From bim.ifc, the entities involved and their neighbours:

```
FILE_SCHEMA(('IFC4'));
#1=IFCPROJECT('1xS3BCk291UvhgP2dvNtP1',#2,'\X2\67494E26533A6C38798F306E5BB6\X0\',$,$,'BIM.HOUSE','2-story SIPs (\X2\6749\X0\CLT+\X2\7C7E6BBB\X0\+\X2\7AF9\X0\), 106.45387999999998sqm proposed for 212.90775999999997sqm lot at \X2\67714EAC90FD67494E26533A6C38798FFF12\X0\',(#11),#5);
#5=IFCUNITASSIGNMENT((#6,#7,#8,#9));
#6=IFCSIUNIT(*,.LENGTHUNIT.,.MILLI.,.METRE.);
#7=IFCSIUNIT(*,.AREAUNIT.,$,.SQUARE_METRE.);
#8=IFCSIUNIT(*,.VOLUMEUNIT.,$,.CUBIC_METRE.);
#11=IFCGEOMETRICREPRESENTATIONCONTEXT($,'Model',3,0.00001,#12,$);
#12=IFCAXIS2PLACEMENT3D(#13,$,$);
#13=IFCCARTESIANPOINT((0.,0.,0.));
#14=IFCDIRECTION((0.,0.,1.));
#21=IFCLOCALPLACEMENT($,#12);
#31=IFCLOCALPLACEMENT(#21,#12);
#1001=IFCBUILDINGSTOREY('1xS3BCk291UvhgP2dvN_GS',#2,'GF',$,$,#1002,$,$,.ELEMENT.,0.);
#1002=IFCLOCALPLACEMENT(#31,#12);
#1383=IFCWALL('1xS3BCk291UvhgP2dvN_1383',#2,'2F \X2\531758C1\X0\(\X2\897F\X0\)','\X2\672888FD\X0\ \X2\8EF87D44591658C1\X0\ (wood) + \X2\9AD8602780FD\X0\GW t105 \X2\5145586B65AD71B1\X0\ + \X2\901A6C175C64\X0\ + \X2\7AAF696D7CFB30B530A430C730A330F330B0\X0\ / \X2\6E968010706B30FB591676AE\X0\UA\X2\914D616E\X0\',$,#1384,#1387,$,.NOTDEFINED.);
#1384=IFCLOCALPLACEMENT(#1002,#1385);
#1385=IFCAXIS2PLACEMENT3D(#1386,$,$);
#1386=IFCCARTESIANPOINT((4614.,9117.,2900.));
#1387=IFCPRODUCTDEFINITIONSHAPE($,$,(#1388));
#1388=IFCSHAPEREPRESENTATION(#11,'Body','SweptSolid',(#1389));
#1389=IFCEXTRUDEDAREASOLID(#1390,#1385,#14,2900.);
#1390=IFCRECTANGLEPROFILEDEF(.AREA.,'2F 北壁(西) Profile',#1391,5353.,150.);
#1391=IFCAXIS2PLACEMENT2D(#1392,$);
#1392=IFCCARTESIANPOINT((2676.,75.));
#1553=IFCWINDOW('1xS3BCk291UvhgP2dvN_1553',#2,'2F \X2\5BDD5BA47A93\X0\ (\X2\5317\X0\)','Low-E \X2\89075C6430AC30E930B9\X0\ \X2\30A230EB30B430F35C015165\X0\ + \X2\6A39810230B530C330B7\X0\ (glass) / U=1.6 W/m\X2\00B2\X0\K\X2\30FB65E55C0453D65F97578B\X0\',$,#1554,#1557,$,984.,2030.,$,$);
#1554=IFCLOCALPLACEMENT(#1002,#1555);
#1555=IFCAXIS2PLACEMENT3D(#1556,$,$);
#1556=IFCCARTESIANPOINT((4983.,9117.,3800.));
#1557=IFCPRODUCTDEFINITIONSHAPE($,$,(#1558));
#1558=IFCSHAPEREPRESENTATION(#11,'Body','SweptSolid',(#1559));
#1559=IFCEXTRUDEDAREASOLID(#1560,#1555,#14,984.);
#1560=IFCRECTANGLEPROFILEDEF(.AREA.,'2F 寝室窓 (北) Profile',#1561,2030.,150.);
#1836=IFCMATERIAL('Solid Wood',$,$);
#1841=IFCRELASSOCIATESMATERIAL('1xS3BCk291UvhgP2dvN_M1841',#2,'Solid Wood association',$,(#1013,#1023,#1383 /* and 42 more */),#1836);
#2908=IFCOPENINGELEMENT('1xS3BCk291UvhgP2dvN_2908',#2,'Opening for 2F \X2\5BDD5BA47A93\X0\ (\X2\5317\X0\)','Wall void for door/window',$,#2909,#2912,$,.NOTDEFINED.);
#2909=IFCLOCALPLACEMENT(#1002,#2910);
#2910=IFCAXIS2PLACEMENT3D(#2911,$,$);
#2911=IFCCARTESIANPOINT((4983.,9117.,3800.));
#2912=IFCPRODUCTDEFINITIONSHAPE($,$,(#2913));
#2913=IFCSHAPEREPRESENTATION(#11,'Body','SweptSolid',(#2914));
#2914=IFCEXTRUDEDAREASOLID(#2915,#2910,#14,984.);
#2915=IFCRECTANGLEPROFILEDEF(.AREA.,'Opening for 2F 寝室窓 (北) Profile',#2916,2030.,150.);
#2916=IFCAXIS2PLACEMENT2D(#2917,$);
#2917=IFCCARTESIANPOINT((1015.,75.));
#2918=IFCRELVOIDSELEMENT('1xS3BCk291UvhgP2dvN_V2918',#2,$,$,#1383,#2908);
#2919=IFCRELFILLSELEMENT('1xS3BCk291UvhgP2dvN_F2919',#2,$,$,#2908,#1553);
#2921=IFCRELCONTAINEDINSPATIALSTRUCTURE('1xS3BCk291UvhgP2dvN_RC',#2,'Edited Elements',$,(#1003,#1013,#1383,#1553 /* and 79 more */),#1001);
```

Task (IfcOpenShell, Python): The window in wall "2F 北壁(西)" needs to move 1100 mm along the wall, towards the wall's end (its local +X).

```python
import ifcopenshell
import ifcopenshell.api.geometry
import ifcopenshell.util.placement
import ifcopenshell.util.unit

model = ifcopenshell.open("bim.ifc")
unit_scale = ifcopenshell.util.unit.calculate_unit_scale(model)

window = model.by_id(1553)
opening = window.FillsVoids[0].RelatingOpeningElement
wall = opening.VoidsElements[0].RelatingBuildingElement

wall_matrix = ifcopenshell.util.placement.get_local_placement(wall.ObjectPlacement)
shift = wall_matrix[:3, 0] * 1.1 / unit_scale
before = ifcopenshell.util.placement.get_local_placement(window.ObjectPlacement)[:3, 3].copy()

# The window is not placed relative to its opening, so move both.
for product in (opening, window):
    matrix = ifcopenshell.util.placement.get_local_placement(product.ObjectPlacement)
    matrix[:3, 3] += shift
    ifcopenshell.api.geometry.edit_object_placement(model, product=product, matrix=matrix, is_si=False)

after = ifcopenshell.util.placement.get_local_placement(window.ObjectPlacement)[:3, 3]
print("window moved by", (after - before).round(3) + 0.0)

model.write("bim-out.ifc")
```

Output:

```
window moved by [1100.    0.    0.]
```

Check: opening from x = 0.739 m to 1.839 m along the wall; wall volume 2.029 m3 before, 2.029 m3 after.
